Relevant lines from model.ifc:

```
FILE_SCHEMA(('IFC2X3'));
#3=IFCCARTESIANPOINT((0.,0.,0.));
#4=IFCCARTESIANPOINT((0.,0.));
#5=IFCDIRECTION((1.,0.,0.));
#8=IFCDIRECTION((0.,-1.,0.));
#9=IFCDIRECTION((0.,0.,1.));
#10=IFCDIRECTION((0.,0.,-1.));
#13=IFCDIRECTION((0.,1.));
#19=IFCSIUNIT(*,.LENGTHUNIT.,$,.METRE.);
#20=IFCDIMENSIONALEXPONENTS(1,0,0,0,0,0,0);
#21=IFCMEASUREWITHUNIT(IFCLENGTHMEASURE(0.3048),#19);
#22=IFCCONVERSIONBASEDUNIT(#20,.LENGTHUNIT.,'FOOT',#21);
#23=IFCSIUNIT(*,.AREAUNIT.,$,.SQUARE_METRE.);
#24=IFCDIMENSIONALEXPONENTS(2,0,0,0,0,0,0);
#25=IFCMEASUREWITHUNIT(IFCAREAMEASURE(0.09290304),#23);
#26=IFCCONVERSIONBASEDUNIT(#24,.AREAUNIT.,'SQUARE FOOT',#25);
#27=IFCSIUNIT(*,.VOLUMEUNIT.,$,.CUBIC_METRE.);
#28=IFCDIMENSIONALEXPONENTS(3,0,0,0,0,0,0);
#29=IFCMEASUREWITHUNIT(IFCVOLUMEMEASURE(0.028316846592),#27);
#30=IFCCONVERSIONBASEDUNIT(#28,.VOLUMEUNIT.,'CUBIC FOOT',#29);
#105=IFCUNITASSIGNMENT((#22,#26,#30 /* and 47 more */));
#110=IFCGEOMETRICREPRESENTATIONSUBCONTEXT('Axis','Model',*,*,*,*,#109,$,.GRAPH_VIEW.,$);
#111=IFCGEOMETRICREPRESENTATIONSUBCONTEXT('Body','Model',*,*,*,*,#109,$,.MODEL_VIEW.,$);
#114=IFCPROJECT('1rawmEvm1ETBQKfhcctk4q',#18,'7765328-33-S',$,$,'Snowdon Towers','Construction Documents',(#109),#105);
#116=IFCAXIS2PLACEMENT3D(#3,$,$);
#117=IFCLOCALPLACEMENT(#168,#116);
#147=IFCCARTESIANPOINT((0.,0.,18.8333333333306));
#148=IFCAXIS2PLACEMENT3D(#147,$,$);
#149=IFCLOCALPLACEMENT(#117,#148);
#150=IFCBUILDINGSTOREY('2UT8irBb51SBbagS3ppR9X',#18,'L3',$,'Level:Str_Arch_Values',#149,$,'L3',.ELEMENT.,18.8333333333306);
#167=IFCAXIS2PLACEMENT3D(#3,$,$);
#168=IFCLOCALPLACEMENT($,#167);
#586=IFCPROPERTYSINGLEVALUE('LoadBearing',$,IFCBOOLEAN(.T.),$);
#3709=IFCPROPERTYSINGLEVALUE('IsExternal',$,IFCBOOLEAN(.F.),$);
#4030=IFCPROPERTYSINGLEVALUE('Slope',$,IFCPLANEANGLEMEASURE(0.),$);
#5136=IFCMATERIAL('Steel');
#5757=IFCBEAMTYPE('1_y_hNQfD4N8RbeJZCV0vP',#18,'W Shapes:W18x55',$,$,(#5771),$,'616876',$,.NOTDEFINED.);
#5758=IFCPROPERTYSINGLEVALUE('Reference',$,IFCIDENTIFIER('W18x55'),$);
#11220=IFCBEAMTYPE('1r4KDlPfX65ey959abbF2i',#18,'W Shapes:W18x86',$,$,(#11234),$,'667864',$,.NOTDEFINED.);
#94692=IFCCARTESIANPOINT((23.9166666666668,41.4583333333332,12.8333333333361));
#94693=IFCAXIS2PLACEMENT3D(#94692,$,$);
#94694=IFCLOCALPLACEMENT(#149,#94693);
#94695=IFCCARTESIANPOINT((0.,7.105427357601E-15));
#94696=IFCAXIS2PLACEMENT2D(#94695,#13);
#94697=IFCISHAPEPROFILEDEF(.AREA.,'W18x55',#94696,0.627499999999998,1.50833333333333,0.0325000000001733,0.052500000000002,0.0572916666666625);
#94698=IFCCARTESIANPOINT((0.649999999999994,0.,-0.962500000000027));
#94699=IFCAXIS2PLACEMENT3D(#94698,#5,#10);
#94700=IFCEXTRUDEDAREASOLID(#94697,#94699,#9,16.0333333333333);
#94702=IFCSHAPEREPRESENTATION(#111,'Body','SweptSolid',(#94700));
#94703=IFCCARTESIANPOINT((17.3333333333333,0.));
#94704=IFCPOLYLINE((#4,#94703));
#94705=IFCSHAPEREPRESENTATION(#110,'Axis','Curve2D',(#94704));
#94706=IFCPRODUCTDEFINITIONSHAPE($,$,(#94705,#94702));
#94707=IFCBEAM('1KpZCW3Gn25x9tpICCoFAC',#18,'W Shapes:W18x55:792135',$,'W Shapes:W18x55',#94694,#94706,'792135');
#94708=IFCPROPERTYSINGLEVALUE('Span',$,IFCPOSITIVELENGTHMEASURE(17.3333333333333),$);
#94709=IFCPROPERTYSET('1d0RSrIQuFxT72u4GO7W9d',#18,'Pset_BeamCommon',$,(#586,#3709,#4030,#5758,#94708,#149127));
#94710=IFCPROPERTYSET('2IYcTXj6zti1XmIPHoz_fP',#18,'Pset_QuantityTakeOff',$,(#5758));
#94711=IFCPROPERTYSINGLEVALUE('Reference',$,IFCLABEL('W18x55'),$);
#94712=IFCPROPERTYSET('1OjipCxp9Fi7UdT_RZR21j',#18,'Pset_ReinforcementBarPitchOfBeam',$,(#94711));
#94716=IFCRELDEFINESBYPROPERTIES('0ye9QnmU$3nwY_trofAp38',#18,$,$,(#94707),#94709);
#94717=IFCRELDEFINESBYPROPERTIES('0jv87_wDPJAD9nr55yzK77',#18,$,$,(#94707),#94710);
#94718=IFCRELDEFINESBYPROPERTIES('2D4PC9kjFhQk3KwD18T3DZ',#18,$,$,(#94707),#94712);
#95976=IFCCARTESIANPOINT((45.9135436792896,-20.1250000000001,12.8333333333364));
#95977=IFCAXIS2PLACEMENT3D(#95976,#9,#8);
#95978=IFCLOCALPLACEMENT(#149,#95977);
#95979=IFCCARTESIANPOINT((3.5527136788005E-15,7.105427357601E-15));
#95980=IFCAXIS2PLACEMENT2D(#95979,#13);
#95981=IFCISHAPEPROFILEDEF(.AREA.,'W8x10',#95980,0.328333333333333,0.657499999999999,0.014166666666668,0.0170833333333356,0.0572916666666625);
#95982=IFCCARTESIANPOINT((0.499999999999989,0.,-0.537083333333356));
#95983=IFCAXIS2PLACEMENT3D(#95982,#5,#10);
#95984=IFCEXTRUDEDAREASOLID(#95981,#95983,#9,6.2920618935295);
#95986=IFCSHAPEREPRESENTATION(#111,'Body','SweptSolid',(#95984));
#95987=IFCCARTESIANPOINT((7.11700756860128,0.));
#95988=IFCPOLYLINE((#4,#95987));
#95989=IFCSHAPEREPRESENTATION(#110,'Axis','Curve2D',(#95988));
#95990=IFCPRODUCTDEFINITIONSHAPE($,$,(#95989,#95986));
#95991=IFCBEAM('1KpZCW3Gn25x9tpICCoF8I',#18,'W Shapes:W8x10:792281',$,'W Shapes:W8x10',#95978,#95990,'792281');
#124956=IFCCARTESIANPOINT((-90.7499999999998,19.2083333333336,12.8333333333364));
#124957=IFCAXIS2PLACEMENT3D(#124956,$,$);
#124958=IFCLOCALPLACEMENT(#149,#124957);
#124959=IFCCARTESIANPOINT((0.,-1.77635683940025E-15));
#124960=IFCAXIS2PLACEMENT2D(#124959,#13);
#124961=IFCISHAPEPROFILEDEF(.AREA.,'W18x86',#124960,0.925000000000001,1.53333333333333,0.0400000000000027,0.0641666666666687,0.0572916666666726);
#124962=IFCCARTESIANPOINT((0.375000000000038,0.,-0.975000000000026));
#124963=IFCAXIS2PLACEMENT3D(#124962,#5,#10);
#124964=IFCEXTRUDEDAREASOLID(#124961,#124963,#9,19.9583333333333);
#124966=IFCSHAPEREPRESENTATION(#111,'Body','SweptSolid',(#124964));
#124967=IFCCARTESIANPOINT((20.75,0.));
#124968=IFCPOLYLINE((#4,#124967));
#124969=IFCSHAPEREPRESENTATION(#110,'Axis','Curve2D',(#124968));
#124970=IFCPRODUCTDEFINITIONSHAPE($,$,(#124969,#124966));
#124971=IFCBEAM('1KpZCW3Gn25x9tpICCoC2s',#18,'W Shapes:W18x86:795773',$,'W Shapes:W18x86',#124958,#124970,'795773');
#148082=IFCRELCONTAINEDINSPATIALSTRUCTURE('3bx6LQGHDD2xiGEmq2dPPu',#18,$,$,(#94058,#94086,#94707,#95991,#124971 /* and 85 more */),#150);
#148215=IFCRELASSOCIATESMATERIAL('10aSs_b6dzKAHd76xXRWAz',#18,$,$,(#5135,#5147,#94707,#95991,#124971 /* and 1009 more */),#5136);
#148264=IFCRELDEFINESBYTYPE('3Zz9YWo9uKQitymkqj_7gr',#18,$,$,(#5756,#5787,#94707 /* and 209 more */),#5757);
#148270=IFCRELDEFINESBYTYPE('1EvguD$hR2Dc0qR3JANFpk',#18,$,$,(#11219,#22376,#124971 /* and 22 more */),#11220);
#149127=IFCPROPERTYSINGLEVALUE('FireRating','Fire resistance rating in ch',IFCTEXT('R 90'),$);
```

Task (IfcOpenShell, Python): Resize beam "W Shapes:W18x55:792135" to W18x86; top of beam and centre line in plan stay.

```python
import ifcopenshell
import ifcopenshell.api.pset
import ifcopenshell.api.type
import ifcopenshell.util.element
import ifcopenshell.util.representation

model = ifcopenshell.open("model.ifc")

member = model.by_guid("1KpZCW3Gn25x9tpICCoFAC")
source = next(p for p in model.by_type("IfcIShapeProfileDef") if p.ProfileName == "W18x86")

body = ifcopenshell.util.representation.get_representation(member, "Model", "Body")
solid = body.Items[0]
old_profile = solid.SweptArea

# Copy the section's sizes but keep this member's own profile position.
profile = ifcopenshell.util.element.copy(model, source)
# Profiles are centred, so shift by half the change in depth to hold the top.
shift = (old_profile.OverallDepth - profile.OverallDepth) / 2
x, y = old_profile.Position.Location.Coordinates
up = (-1.0, 0.0)  # upwards, in the solid's own plane
location = model.createIfcCartesianPoint((x + up[0] * shift, y + up[1] * shift))
profile.Position = model.createIfcAxis2Placement2D(location, old_profile.Position.RefDirection)
solid.SweptArea = profile
if not model.get_total_inverses(old_profile):
    ifcopenshell.util.element.remove_deep2(model, old_profile)

new_type = model.by_guid("1r4KDlPfX65ey959abbF2i")
ifcopenshell.api.type.assign_type(
    model, related_objects=[member], relating_type=new_type, should_map_representations=False
)
member.Name = member.Name.replace("W18x55", "W18x86")
member.ObjectType = "W Shapes:W18x86"
pset = model.by_id(ifcopenshell.util.element.get_pset(member, "Pset_BeamCommon", should_inherit=False)["id"])
ifcopenshell.api.pset.edit_pset(model, pset=pset, properties={"Reference": "W18x86"})
pset = model.by_id(ifcopenshell.util.element.get_pset(member, "Pset_QuantityTakeOff", should_inherit=False)["id"])
ifcopenshell.api.pset.edit_pset(model, pset=pset, properties={"Reference": "W18x86"})
pset = model.by_id(ifcopenshell.util.element.get_pset(member, "Pset_ReinforcementBarPitchOfBeam", should_inherit=False)["id"])
ifcopenshell.api.pset.edit_pset(model, pset=pset, properties={"Reference": "W18x86"})

print(solid.SweptArea)

model.write("model_rev.ifc")
```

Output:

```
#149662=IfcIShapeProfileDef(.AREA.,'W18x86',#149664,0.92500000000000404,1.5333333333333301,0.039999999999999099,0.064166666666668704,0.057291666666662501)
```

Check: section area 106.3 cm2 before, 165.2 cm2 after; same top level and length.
